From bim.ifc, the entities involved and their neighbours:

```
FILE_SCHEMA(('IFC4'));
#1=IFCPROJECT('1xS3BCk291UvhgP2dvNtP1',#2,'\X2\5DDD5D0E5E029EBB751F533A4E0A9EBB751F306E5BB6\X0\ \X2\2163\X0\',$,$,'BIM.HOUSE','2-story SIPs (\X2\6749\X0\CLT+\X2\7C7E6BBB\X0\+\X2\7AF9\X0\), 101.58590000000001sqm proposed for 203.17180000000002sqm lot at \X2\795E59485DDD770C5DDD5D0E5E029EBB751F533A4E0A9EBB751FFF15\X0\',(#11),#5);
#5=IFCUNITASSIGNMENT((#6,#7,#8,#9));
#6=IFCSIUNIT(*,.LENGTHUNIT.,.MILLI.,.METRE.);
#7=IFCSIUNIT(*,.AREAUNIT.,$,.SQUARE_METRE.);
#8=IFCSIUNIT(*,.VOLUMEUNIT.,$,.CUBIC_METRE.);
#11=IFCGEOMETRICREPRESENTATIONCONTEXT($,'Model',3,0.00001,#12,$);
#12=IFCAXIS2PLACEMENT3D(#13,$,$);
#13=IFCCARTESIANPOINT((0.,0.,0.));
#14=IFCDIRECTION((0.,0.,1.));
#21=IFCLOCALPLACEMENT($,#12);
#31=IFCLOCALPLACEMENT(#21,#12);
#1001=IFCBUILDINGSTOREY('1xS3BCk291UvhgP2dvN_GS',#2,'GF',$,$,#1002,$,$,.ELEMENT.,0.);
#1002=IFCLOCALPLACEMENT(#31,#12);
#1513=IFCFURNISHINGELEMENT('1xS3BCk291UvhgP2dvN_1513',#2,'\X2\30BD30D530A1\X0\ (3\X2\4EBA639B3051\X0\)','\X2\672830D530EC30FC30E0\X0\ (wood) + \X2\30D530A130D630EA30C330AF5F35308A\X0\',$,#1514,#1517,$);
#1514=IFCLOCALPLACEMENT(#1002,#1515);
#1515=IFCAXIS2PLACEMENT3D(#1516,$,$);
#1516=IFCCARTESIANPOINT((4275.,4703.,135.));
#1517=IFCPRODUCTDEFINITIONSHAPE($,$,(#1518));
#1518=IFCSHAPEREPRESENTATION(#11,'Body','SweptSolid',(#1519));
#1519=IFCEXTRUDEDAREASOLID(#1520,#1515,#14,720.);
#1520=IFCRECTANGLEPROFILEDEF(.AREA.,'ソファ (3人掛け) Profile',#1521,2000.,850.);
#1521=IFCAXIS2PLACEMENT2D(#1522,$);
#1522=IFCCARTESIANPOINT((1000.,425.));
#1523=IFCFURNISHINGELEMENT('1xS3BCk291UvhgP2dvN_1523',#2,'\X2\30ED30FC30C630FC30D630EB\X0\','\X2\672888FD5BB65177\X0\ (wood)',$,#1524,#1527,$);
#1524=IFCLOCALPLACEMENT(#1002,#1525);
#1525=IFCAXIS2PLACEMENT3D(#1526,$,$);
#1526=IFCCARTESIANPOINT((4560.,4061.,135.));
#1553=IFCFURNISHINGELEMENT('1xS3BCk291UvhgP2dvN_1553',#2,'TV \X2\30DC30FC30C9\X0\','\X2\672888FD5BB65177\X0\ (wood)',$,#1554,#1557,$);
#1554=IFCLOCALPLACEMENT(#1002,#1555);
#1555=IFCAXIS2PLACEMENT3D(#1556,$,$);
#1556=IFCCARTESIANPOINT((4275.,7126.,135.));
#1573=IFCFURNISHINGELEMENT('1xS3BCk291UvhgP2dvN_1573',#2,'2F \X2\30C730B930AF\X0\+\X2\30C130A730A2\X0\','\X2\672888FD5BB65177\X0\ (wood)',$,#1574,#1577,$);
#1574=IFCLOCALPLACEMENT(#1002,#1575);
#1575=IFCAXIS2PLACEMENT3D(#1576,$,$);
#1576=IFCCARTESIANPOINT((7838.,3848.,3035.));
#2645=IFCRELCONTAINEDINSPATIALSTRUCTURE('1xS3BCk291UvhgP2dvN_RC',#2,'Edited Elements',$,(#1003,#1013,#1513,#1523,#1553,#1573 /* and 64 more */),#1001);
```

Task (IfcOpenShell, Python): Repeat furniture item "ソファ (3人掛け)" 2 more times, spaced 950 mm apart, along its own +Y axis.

```python
import ifcopenshell
import ifcopenshell.api.geometry
import ifcopenshell.api.root
import ifcopenshell.util.element
import ifcopenshell.util.placement
import ifcopenshell.util.unit

model = ifcopenshell.open("bim.ifc")
unit_scale = ifcopenshell.util.unit.calculate_unit_scale(model)


def reuse_history(source, copy):
    """copy_class also copies each property set's owner history, people and application; keep the originals."""
    for rel in copy.IsDefinedBy:
        if rel.is_a("IfcRelDefinesByProperties") and (history := rel.RelatingPropertyDefinition.OwnerHistory):
            rel.RelatingPropertyDefinition.OwnerHistory = source.OwnerHistory
            ifcopenshell.util.element.remove_deep2(model, history)


source = model.by_id(1513)
base = ifcopenshell.util.placement.get_local_placement(source.ObjectPlacement)
step = base[:3, 1] * 0.95 / unit_scale

for i in range(1, 3):
    copy = ifcopenshell.api.root.copy_class(model, product=source)
    copy.Representation = ifcopenshell.util.element.copy_deep(
        model, source.Representation, exclude=["IfcGeometricRepresentationContext", "IfcRepresentationMap"]
    )
    reuse_history(source, copy)
    matrix = base.copy()
    matrix[:3, 3] += i * step
    print("added at", matrix[:3, 3].round(3) + 0.0)
    ifcopenshell.api.geometry.edit_object_placement(model, product=copy, matrix=matrix, is_si=False)

model.write("bim_rev.ifc")
```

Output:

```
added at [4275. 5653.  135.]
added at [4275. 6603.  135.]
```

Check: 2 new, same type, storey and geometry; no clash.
